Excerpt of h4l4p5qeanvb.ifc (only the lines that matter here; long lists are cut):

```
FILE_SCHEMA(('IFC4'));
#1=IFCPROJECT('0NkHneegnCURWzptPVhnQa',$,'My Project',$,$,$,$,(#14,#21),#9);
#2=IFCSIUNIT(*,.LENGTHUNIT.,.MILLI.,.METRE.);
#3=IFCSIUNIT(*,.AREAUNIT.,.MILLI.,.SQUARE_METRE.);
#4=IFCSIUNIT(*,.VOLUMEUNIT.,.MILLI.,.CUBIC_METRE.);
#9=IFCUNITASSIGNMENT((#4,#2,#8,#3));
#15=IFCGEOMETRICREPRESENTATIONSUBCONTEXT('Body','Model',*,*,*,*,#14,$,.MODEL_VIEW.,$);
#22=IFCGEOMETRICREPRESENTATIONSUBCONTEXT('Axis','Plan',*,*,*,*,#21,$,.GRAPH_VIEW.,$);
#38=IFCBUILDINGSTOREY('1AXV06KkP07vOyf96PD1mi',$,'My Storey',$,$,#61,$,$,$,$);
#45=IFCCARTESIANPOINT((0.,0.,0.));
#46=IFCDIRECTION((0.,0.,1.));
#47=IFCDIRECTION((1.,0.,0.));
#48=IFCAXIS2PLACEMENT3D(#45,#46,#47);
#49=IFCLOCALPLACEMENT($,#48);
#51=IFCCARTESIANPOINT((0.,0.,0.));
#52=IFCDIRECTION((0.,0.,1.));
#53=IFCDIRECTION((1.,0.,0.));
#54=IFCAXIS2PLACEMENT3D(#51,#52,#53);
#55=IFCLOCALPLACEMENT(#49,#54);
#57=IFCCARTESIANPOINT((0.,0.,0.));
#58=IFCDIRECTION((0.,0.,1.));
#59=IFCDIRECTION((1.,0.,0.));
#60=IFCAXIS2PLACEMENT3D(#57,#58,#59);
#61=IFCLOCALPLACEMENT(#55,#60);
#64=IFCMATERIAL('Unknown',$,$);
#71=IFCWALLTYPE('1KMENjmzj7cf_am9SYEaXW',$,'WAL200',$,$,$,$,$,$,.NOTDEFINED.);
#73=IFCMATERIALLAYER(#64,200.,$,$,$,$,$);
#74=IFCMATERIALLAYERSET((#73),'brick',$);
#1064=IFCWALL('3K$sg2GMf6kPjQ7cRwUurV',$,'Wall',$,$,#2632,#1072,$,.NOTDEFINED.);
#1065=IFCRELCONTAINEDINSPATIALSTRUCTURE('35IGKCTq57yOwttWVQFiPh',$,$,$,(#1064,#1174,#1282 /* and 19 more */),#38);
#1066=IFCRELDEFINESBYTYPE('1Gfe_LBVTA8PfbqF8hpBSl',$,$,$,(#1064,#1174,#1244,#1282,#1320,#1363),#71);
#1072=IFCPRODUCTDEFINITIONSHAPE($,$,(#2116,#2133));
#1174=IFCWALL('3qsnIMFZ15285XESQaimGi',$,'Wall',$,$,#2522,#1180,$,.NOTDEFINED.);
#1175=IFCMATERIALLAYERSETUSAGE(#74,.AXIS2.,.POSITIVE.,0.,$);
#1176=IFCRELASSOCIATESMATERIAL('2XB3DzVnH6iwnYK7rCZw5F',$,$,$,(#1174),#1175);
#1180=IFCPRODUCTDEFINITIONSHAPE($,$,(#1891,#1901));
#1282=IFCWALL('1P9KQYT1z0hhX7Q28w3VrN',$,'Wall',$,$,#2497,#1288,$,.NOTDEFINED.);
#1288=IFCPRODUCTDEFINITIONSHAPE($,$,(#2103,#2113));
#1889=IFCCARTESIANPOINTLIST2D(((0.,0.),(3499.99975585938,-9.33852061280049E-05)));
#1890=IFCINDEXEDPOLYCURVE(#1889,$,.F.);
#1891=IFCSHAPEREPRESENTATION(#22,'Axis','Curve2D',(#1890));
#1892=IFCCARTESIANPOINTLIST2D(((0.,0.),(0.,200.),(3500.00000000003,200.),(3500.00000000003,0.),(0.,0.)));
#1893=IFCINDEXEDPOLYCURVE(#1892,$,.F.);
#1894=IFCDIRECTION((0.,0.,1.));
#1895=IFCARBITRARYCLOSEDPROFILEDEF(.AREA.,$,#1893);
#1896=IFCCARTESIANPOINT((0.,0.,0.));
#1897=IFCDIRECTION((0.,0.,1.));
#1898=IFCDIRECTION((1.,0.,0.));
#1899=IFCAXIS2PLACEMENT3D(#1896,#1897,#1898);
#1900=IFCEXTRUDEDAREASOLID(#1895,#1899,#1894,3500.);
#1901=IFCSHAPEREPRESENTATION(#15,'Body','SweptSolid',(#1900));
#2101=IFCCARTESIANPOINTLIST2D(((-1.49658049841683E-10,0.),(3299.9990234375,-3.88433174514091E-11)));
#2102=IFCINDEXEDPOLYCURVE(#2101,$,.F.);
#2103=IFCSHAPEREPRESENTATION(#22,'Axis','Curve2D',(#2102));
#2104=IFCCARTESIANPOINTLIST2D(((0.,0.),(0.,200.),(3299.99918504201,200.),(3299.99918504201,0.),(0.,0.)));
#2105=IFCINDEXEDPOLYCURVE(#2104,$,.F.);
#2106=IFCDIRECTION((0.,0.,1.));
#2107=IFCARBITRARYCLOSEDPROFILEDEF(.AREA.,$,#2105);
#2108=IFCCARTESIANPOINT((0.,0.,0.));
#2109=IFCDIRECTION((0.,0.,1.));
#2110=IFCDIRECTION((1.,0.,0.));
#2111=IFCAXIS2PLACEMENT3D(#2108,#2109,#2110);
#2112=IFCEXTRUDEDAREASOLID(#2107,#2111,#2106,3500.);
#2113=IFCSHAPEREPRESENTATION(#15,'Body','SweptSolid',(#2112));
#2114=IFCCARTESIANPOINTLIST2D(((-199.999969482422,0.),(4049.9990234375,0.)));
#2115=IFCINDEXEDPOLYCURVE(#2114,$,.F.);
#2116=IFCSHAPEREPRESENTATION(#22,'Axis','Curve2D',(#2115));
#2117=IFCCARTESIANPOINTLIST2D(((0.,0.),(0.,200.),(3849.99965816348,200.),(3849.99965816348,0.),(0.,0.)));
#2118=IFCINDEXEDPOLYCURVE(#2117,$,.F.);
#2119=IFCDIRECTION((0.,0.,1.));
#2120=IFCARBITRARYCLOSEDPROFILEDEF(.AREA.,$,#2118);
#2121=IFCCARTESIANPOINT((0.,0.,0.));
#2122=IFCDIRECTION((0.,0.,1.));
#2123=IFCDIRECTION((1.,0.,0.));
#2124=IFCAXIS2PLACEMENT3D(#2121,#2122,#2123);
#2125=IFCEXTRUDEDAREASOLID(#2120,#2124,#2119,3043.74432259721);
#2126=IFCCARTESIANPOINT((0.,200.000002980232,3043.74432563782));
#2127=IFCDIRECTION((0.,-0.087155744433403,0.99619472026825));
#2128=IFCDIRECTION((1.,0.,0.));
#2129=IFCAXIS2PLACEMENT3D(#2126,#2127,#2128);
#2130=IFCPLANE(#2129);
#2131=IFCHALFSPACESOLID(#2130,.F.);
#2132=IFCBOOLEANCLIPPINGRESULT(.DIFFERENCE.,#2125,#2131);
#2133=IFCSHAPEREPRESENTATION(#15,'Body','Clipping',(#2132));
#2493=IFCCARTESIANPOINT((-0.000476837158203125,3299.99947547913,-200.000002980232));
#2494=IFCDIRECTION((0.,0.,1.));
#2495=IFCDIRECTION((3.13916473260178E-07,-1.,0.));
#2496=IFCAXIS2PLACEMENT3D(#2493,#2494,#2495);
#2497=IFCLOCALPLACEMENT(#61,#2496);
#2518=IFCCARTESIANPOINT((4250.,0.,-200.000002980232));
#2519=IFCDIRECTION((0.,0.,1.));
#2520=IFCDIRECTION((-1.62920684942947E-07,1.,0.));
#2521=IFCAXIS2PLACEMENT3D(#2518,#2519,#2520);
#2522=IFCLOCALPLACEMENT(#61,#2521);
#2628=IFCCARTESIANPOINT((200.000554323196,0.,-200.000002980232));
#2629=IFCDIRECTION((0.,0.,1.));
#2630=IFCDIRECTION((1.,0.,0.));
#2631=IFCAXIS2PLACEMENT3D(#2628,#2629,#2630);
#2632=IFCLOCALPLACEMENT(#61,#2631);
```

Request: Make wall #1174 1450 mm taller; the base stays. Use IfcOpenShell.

```python
import ifcopenshell
import ifcopenshell.geom
import ifcopenshell.util.representation
import ifcopenshell.util.shape
import ifcopenshell.util.unit

model = ifcopenshell.open("h4l4p5qeanvb.ifc")
unit_scale = ifcopenshell.util.unit.calculate_unit_scale(model)
settings = ifcopenshell.geom.settings()


def volume(element):
    """Net volume in cubic metres, openings subtracted."""
    shape = ifcopenshell.geom.create_shape(settings, element)
    return ifcopenshell.util.shape.get_volume(shape.geometry)


wall = model.by_guid("3qsnIMFZ15285XESQaimGi")
before = volume(wall)

body = ifcopenshell.util.representation.get_representation(wall, "Model", "Body")
solid = body.Items[0]
old_height = solid.Depth
solid.Depth += 1.45 / unit_scale
after = volume(wall)

print(f"height {old_height:g} -> {solid.Depth:g}, volume {before:.3f} -> {after:.3f} m3")

model.write("h4l4p5qeanvb_updated.ifc")
```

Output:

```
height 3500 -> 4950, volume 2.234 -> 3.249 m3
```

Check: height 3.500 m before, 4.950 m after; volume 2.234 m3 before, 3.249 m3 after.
